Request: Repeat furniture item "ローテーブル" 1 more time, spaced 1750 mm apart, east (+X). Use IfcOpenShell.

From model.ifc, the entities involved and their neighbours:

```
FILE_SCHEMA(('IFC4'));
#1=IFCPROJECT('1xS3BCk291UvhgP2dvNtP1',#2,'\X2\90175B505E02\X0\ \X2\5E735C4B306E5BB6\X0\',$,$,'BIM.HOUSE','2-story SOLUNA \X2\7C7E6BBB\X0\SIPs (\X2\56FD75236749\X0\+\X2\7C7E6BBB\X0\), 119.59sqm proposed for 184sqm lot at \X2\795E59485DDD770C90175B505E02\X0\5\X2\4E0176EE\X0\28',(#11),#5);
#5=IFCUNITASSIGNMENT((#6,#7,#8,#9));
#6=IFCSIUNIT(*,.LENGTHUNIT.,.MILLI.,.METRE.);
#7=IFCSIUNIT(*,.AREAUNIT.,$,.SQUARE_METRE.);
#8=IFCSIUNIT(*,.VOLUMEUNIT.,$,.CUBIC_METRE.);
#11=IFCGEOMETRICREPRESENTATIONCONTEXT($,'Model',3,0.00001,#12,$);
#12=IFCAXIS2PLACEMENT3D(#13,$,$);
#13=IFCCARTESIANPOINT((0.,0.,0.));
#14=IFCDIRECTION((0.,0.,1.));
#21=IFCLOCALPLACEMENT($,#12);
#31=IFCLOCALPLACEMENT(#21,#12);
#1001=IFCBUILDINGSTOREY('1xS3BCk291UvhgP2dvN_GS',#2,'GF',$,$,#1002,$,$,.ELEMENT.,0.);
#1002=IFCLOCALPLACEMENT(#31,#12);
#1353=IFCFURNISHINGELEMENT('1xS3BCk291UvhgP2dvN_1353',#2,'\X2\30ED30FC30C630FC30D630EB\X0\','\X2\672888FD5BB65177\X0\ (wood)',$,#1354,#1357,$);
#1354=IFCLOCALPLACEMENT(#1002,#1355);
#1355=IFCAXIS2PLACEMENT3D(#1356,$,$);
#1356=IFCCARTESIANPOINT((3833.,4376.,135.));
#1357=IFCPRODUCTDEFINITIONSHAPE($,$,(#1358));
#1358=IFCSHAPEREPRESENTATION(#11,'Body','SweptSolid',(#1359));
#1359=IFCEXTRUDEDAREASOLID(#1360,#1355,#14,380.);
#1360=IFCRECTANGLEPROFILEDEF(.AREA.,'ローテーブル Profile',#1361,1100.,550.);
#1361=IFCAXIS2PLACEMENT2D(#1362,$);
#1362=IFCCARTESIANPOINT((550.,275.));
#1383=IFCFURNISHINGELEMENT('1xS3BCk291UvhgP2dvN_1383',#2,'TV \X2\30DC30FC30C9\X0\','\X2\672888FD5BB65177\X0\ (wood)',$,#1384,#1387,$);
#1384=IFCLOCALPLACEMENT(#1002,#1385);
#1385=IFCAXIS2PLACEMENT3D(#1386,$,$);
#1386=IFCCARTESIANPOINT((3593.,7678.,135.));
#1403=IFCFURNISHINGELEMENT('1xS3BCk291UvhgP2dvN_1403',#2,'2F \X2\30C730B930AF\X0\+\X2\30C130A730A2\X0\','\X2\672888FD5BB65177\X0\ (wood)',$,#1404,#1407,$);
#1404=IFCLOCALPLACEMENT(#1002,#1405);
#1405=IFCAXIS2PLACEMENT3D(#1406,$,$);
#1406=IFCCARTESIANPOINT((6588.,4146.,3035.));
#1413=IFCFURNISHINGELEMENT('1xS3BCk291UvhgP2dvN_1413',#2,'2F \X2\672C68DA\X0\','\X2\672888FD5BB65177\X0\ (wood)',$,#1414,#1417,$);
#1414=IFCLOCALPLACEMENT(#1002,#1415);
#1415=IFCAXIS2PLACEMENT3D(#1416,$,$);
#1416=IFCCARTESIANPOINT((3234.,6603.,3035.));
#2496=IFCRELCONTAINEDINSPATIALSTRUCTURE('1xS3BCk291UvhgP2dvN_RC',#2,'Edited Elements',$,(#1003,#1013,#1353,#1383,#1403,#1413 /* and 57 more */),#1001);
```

```python
import numpy as np
import ifcopenshell
import ifcopenshell.api.geometry
import ifcopenshell.api.root
import ifcopenshell.util.element
import ifcopenshell.util.placement

model = ifcopenshell.open("model.ifc")


def reuse_history(source, copy):
    """copy_class also copies each property set's owner history, people and application; keep the originals."""
    for rel in copy.IsDefinedBy:
        if rel.is_a("IfcRelDefinesByProperties") and (history := rel.RelatingPropertyDefinition.OwnerHistory):
            rel.RelatingPropertyDefinition.OwnerHistory = source.OwnerHistory
            ifcopenshell.util.element.remove_deep2(model, history)


source = model.by_guid("1xS3BCk291UvhgP2dvN_1353")
base = ifcopenshell.util.placement.get_local_placement(source.ObjectPlacement)
step = np.array([1.0, 0.0, 0.0]) * 1750.0

for i in range(1, 2):
    copy = ifcopenshell.api.root.copy_class(model, product=source)
    copy.Representation = ifcopenshell.util.element.copy_deep(
        model, source.Representation, exclude=["IfcGeometricRepresentationContext", "IfcRepresentationMap"]
    )
    reuse_history(source, copy)
    matrix = base.copy()
    matrix[:3, 3] += i * step
    print("added at", matrix[:3, 3].round(3) + 0.0)
    ifcopenshell.api.geometry.edit_object_placement(model, product=copy, matrix=matrix, is_si=False)

model.write("model_rev.ifc")
```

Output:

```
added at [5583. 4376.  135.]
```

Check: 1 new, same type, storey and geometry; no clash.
